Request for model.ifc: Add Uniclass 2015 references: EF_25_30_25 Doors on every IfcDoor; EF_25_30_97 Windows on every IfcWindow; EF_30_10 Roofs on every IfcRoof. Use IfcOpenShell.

First a look at what the model holds.

```python
import ifcopenshell

model = ifcopenshell.open("model.ifc")
print(model.schema)
print("classifications:", [c.Name for c in model.by_type("IfcClassification")])
for ifc_class in ("IfcDoor", "IfcRoof", "IfcStair", "IfcWall", "IfcWindow"):
    print(ifc_class, len(model.by_type(ifc_class)))
```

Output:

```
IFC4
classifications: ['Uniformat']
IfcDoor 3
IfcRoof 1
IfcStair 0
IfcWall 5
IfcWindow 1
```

```python
import ifcopenshell
import ifcopenshell.api.classification

model = ifcopenshell.open("model.ifc")

system = ifcopenshell.api.classification.add_classification(model, classification="Uniclass 2015")

codes = {
    "IfcDoor": ("EF_25_30_25", "Doors"),
    "IfcWindow": ("EF_25_30_97", "Windows"),
    "IfcRoof": ("EF_30_10", "Roofs"),
}
for ifc_class, (code, name) in codes.items():
    products = model.by_type(ifc_class)
    ifcopenshell.api.classification.add_reference(
        model, products=products, classification=system, identification=code, name=name
    )
    print(code, len(products))

model.write("model-out.ifc")
```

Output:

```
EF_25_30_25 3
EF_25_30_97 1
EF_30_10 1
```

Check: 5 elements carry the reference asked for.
